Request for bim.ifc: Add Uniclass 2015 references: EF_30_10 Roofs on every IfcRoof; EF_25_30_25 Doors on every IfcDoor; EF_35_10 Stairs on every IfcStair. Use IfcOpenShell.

First a look at what the model holds.

```python
import ifcopenshell

model = ifcopenshell.open("bim.ifc")
print(model.schema)
print("classifications:", [c.Name for c in model.by_type("IfcClassification")])
for ifc_class in ("IfcDoor", "IfcRoof", "IfcStair", "IfcWall", "IfcWindow"):
    print(ifc_class, len(model.by_type(ifc_class)))
```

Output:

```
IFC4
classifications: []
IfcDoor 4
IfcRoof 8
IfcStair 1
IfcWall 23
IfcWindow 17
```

```python
import ifcopenshell
import ifcopenshell.api.classification

model = ifcopenshell.open("bim.ifc")

system = ifcopenshell.api.classification.add_classification(model, classification="Uniclass 2015")

codes = {
    "IfcRoof": ("EF_30_10", "Roofs"),
    "IfcDoor": ("EF_25_30_25", "Doors"),
    "IfcStair": ("EF_35_10", "Stairs"),
}
for ifc_class, (code, name) in codes.items():
    products = model.by_type(ifc_class)
    ifcopenshell.api.classification.add_reference(
        model, products=products, classification=system, identification=code, name=name
    )
    print(code, len(products))

model.write("bim_rev.ifc")
```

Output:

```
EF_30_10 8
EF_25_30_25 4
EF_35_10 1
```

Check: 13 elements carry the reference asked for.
